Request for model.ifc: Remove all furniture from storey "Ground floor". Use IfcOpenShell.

First a look at what the model holds.

```python
import ifcopenshell
import ifcopenshell.util.element

model = ifcopenshell.open("model.ifc")
print(model.schema)
storey = next(s for s in model.by_type("IfcBuildingStorey") if s.Name == "Ground floor")
furniture = [e for e in ifcopenshell.util.element.get_decomposition(storey) if e.is_a("IfcFurnishingElement")]
seen = {}
for e in furniture:
    element_type = ifcopenshell.util.element.get_type(e)
    name = element_type.Name if element_type not in (None, e) else None
    seen[name] = seen.get(name, 0) + 1
for name, count in sorted(seen.items(), key=str):
    print(count, "x", name)
```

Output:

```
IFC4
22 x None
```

```python
import ifcopenshell
import ifcopenshell.api.root
import ifcopenshell.util.element

model = ifcopenshell.open("model.ifc")

storey = next(s for s in model.by_type("IfcBuildingStorey") if s.Name == "Ground floor")
furniture = [e for e in ifcopenshell.util.element.get_decomposition(storey) if e.is_a("IfcFurnishingElement")]

for e in furniture:
    ifcopenshell.api.root.remove_product(model, product=e)
print(len(furniture), "removed")

model.write("model-out.ifc")
```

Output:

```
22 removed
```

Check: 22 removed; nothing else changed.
